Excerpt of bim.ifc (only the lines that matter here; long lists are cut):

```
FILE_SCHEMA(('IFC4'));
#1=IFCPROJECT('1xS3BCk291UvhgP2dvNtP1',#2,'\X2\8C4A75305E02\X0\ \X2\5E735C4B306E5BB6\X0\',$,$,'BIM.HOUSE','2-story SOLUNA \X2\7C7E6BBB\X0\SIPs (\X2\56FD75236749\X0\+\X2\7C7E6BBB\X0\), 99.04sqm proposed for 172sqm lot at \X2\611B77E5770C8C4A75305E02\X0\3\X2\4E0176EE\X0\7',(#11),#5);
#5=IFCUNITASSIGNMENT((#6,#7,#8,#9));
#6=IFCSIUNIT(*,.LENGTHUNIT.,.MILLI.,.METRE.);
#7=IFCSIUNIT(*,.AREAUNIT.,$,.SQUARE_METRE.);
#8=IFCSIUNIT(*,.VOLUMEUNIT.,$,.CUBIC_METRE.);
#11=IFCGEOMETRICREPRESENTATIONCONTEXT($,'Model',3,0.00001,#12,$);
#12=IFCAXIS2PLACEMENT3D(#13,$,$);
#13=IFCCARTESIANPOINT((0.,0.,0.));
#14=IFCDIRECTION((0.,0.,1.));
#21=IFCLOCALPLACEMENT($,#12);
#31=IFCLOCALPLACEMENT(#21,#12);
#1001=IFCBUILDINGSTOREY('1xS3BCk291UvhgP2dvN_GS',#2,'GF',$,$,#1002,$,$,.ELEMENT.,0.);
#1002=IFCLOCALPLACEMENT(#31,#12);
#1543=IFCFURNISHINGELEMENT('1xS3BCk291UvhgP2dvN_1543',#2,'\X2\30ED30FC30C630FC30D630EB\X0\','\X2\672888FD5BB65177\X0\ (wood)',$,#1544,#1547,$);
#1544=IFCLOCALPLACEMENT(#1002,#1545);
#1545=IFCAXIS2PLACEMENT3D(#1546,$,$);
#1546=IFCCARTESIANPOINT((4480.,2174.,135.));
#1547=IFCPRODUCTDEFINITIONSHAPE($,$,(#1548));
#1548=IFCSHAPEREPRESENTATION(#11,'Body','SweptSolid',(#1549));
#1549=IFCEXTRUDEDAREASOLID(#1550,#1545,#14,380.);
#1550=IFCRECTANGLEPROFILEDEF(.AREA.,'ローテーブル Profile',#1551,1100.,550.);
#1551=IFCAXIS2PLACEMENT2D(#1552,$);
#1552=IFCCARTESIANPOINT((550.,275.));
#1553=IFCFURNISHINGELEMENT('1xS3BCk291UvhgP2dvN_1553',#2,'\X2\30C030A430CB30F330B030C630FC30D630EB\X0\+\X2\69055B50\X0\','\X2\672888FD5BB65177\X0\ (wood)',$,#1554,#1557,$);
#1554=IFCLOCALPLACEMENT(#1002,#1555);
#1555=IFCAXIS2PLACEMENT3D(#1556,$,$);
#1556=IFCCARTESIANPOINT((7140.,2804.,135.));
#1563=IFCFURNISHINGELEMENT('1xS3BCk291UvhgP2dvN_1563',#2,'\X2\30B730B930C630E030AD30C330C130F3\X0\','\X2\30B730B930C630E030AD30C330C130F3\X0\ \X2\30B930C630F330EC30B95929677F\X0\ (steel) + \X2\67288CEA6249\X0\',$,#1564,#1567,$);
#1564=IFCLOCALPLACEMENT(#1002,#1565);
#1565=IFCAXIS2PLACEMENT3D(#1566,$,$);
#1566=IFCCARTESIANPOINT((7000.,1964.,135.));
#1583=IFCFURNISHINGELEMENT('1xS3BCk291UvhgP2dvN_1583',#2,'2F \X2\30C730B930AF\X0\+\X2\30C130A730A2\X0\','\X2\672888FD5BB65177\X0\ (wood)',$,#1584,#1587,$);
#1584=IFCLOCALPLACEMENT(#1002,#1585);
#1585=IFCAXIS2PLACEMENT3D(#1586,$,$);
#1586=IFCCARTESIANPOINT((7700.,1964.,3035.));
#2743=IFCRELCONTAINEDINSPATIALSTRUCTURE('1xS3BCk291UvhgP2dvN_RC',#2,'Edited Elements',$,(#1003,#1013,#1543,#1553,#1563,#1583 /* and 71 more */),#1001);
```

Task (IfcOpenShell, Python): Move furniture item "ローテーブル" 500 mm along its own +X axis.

```python
import ifcopenshell
import ifcopenshell.api.geometry
import ifcopenshell.util.placement
import ifcopenshell.util.unit

model = ifcopenshell.open("bim.ifc")
unit_scale = ifcopenshell.util.unit.calculate_unit_scale(model)

item = model.by_guid("1xS3BCk291UvhgP2dvN_1543")
matrix = ifcopenshell.util.placement.get_local_placement(item.ObjectPlacement)
matrix[:3, 3] += matrix[:3, 0] * 0.5 / unit_scale
ifcopenshell.api.geometry.edit_object_placement(model, product=item, matrix=matrix, is_si=False)

print(ifcopenshell.util.placement.get_local_placement(item.ObjectPlacement).round(3) + 0.0)

model.write("bim-out.ifc")
```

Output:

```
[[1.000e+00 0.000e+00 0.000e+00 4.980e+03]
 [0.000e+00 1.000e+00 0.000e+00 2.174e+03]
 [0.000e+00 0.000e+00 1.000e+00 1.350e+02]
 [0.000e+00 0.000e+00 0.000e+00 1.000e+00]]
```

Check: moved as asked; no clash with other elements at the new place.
